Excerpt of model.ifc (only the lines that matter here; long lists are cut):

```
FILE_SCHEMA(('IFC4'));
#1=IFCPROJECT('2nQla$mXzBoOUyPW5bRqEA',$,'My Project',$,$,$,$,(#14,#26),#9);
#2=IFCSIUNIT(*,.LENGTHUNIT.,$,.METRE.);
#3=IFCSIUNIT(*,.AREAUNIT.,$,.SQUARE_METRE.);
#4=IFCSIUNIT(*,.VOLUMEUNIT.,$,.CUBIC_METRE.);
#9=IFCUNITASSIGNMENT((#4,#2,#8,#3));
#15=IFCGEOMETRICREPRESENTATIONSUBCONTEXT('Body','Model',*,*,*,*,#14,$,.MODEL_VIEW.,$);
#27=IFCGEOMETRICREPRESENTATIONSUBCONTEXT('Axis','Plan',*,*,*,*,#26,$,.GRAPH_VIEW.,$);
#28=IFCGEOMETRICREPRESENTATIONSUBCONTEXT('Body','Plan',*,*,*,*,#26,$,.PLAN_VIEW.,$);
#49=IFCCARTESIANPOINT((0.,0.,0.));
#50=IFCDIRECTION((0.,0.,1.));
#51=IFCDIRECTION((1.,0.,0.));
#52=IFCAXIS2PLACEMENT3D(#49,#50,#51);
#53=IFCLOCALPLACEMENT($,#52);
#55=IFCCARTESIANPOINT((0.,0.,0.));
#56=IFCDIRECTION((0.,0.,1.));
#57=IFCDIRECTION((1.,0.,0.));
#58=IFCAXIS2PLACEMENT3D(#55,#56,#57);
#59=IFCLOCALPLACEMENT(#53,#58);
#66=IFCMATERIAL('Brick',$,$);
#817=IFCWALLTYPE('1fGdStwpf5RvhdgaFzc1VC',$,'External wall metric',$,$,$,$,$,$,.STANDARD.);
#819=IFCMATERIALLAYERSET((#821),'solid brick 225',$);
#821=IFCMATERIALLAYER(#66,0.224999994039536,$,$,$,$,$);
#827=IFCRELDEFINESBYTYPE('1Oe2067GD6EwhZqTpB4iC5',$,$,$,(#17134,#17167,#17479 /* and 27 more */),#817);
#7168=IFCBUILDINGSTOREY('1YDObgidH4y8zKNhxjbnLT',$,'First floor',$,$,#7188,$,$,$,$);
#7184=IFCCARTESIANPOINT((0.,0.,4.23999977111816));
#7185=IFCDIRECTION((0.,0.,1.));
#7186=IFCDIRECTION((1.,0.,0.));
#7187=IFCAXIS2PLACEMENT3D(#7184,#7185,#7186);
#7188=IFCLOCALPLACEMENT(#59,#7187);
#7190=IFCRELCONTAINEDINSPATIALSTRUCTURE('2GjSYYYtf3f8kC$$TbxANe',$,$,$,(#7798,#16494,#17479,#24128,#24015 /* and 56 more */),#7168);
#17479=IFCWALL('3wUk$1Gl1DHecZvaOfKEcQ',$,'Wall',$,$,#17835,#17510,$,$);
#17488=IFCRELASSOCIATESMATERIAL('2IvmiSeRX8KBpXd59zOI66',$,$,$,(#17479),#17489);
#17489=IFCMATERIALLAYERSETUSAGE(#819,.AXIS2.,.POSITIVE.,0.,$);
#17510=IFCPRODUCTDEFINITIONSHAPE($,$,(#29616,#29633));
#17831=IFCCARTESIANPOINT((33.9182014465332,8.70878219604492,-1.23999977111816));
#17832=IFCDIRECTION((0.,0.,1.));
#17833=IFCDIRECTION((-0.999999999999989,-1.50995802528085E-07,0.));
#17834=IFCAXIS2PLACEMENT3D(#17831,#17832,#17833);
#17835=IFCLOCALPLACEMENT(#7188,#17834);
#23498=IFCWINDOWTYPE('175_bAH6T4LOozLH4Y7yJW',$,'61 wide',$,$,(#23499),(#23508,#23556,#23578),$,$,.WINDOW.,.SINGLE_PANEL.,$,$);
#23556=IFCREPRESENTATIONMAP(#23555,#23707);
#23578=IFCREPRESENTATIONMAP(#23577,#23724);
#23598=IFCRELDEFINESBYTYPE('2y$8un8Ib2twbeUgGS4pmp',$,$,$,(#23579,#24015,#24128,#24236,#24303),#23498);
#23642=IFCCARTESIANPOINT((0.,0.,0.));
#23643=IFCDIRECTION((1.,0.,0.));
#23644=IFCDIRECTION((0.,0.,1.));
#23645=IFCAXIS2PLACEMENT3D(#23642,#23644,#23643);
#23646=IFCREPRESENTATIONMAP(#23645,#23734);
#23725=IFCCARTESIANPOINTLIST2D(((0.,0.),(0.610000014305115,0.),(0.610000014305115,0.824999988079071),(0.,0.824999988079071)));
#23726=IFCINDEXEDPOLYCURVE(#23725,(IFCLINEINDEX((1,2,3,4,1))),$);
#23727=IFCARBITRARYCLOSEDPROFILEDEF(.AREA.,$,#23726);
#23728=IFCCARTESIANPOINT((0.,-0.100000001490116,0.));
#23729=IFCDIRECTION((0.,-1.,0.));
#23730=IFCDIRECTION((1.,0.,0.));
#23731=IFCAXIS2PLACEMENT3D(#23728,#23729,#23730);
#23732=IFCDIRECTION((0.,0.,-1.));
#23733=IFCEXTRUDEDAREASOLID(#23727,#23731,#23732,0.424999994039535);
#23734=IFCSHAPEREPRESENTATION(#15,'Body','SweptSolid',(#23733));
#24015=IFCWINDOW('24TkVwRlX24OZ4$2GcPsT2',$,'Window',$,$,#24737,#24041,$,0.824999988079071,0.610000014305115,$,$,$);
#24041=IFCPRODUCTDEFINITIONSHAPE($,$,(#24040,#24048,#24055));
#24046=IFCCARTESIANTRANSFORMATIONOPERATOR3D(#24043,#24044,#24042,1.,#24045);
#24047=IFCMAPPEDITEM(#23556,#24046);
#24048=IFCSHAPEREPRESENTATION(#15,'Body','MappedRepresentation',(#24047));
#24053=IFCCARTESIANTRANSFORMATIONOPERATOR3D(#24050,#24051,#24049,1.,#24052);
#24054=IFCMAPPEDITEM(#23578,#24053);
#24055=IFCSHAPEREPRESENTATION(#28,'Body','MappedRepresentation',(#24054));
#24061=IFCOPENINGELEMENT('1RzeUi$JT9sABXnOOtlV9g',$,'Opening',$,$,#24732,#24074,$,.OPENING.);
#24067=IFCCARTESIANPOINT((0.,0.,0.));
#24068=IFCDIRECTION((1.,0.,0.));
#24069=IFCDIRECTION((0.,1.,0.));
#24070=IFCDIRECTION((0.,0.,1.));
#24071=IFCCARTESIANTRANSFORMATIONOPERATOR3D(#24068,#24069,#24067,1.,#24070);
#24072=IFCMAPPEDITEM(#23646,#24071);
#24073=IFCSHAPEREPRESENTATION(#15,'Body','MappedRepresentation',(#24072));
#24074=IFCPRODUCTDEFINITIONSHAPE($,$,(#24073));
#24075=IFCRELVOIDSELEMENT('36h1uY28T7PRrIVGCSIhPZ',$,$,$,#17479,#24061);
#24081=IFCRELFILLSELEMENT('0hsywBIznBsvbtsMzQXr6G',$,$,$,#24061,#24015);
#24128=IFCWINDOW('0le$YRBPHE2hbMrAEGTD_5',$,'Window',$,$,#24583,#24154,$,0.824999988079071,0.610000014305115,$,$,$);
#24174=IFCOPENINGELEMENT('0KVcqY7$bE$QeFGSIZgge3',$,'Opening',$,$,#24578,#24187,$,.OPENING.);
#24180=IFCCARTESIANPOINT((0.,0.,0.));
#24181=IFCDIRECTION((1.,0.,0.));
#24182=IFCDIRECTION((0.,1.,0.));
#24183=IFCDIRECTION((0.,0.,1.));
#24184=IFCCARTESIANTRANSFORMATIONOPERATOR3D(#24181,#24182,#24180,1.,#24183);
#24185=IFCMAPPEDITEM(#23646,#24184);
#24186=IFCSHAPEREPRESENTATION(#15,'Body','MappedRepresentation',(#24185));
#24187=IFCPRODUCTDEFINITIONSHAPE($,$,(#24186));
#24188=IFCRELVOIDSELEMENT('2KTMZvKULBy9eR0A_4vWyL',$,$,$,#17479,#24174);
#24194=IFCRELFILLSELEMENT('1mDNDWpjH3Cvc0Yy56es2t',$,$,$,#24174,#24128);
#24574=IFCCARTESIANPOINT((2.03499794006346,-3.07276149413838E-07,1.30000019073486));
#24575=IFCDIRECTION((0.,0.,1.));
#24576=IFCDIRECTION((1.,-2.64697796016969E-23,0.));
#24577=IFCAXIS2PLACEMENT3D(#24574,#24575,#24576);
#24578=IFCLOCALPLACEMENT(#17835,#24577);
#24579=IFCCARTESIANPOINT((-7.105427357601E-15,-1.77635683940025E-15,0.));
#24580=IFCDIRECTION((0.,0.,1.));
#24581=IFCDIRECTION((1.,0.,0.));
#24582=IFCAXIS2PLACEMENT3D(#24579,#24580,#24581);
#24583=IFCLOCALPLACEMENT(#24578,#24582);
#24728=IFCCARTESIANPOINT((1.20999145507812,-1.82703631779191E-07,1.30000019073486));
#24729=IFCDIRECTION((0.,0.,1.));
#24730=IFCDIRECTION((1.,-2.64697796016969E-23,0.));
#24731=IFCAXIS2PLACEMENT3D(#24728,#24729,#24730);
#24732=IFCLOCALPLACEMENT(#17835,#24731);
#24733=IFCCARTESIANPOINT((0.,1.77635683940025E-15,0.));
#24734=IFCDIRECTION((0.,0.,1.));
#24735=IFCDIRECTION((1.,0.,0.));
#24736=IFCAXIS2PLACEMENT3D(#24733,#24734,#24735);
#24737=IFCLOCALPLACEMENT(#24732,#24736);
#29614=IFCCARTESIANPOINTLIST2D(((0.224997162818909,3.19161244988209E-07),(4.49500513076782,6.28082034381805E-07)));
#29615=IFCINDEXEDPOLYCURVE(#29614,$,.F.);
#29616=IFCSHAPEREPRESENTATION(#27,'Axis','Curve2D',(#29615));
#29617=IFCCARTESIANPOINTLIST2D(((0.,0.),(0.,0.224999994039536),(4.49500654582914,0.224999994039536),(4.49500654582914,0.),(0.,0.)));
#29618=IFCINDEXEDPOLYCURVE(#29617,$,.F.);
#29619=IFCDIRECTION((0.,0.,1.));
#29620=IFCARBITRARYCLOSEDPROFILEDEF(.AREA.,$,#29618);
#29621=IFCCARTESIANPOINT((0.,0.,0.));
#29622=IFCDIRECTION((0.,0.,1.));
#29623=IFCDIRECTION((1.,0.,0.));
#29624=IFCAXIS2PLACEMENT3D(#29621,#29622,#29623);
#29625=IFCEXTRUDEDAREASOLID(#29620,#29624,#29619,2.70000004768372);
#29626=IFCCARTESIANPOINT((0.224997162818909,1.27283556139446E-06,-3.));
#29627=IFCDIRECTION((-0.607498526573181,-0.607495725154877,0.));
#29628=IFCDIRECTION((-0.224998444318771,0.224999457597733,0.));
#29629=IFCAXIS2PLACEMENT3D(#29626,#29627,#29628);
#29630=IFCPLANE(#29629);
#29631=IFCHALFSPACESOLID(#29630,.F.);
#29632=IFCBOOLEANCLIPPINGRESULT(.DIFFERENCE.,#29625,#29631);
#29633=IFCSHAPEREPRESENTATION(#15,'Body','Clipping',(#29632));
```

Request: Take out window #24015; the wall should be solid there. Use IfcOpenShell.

```python
import ifcopenshell
import ifcopenshell.api.feature
import ifcopenshell.api.root
import ifcopenshell.geom
import ifcopenshell.util.shape

model = ifcopenshell.open("model.ifc")
settings = ifcopenshell.geom.settings()


def volume(element):
    """Net volume in cubic metres, openings subtracted."""
    shape = ifcopenshell.geom.create_shape(settings, element)
    return ifcopenshell.util.shape.get_volume(shape.geometry)


window = model.by_guid("24TkVwRlX24OZ4$2GcPsT2")
opening = window.FillsVoids[0].RelatingOpeningElement
wall = opening.VoidsElements[0].RelatingBuildingElement
before = volume(wall)

ifcopenshell.api.root.remove_product(model, product=window)
ifcopenshell.api.feature.remove_feature(model, feature=opening)

after = volume(wall)

print(f"wall volume {before:.3f} -> {after:.3f} m3")

model.write("model-out.ifc")
```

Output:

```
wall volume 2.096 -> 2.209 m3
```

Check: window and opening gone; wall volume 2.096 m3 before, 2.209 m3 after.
